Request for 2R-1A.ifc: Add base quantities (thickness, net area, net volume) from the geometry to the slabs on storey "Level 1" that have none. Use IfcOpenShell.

First a look at what the model holds.

```python
import ifcopenshell
import ifcopenshell.util.element
import ifcopenshell.util.unit

model = ifcopenshell.open("2R-1A.ifc")
print(model.schema)
for unit_type in ("LENGTHUNIT", "AREAUNIT", "VOLUMEUNIT"):
    print(unit_type, ifcopenshell.util.unit.calculate_unit_scale(model, unit_type))
storey = next(s for s in model.by_type("IfcBuildingStorey") if s.Name == "Level 1")
slabs = [e for e in ifcopenshell.util.element.get_decomposition(storey) if e.is_a("IfcSlab")]
for e in sorted(slabs, key=lambda e: e.id()):
    print(e.id(), e.is_a(), e.Name, list(ifcopenshell.util.element.get_psets(e, qtos_only=True)), sep=" | ")
```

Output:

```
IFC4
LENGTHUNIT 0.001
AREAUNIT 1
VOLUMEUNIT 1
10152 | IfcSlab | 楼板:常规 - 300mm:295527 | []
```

```python
import ifcopenshell
import ifcopenshell.api.pset
import ifcopenshell.geom
import ifcopenshell.util.element
import ifcopenshell.util.shape
import ifcopenshell.util.unit

model = ifcopenshell.open("2R-1A.ifc")
unit_scale = ifcopenshell.util.unit.calculate_unit_scale(model)
area_scale = ifcopenshell.util.unit.calculate_unit_scale(model, "AREAUNIT")
volume_scale = ifcopenshell.util.unit.calculate_unit_scale(model, "VOLUMEUNIT")
settings = ifcopenshell.geom.settings()

storey = next(s for s in model.by_type("IfcBuildingStorey") if s.Name == "Level 1")
slabs = [e for e in ifcopenshell.util.element.get_decomposition(storey) if e.is_a("IfcSlab")]

for e in sorted(slabs, key=lambda e: e.id()):
    if ifcopenshell.util.element.get_psets(e, qtos_only=True, should_inherit=False):
        continue
    # Geometry comes back in metres, in the element's own axes.
    shape = ifcopenshell.geom.create_shape(settings, e)
    values = {
        "Width": ifcopenshell.util.shape.get_z(shape.geometry) / unit_scale,
        "NetArea": ifcopenshell.util.shape.get_footprint_area(shape.geometry) / area_scale,
        "NetVolume": ifcopenshell.util.shape.get_volume(shape.geometry) / volume_scale,
    }
    qto = ifcopenshell.api.pset.add_qto(model, product=e, name="Qto_SlabBaseQuantities")
    ifcopenshell.api.pset.edit_qto(model, qto=qto, properties=values)
    print(e.id(), {k: round(v, 3) for k, v in values.items()})

model.write("2R-1A_edited.ifc")
```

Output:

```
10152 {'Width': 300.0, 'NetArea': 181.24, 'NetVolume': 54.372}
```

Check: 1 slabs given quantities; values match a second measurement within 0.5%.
